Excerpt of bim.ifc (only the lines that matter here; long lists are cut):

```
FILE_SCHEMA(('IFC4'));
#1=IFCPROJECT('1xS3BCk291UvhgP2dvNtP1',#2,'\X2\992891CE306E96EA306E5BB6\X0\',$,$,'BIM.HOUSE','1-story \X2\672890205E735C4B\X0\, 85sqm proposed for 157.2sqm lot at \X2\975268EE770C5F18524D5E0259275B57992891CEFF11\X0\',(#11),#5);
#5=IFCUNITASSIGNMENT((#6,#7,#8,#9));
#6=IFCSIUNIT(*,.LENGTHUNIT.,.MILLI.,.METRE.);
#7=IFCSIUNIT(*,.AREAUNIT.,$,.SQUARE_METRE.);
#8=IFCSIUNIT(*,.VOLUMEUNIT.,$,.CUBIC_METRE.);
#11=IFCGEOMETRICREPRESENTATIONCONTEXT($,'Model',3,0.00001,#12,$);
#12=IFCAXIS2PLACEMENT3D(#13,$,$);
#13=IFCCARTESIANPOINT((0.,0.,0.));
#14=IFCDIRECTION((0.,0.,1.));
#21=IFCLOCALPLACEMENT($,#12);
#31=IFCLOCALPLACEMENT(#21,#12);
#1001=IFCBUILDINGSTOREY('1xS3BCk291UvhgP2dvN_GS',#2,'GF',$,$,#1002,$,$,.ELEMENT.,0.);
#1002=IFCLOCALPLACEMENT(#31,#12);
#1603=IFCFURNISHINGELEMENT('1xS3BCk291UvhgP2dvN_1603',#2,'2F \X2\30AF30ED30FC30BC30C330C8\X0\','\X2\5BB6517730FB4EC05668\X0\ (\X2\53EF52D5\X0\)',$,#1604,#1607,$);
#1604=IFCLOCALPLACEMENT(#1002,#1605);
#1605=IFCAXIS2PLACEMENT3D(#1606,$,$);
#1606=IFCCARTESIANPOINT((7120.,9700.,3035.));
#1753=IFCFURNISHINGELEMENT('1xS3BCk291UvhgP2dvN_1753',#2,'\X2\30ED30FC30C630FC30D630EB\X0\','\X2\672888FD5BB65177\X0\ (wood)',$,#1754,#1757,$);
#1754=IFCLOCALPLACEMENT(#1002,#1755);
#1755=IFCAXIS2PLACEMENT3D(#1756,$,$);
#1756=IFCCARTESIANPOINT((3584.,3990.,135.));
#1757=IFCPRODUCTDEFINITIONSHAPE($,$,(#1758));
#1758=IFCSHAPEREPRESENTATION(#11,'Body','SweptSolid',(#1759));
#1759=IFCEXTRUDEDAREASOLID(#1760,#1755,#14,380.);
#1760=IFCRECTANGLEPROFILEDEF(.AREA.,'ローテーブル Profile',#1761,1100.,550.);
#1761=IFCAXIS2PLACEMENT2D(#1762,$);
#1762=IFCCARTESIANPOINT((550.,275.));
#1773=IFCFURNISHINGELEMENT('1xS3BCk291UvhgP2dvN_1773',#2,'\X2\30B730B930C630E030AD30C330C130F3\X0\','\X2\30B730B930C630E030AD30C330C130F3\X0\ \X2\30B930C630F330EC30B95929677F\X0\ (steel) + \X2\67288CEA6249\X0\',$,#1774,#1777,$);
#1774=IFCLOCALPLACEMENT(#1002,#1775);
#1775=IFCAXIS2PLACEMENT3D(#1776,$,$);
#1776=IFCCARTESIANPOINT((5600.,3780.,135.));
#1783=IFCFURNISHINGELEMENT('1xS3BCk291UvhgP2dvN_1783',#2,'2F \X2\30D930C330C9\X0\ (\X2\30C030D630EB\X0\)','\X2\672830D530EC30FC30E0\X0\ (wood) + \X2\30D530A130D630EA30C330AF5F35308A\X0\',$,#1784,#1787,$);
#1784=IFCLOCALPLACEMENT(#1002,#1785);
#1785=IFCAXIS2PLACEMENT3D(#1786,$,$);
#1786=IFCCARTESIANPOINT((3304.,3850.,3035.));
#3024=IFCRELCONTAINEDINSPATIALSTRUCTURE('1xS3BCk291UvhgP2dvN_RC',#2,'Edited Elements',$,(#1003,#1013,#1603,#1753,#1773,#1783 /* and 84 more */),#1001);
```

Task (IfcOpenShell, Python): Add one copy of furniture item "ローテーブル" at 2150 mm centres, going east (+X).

```python
import numpy as np
import ifcopenshell
import ifcopenshell.api.geometry
import ifcopenshell.api.root
import ifcopenshell.util.element
import ifcopenshell.util.placement

model = ifcopenshell.open("bim.ifc")


def reuse_history(source, copy):
    """copy_class also copies each property set's owner history, people and application; keep the originals."""
    for rel in copy.IsDefinedBy:
        if rel.is_a("IfcRelDefinesByProperties") and (history := rel.RelatingPropertyDefinition.OwnerHistory):
            rel.RelatingPropertyDefinition.OwnerHistory = source.OwnerHistory
            ifcopenshell.util.element.remove_deep2(model, history)


source = model.by_id(1753)
base = ifcopenshell.util.placement.get_local_placement(source.ObjectPlacement)
step = np.array([1.0, 0.0, 0.0]) * 2150.0

for i in range(1, 2):
    copy = ifcopenshell.api.root.copy_class(model, product=source)
    copy.Representation = ifcopenshell.util.element.copy_deep(
        model, source.Representation, exclude=["IfcGeometricRepresentationContext", "IfcRepresentationMap"]
    )
    reuse_history(source, copy)
    matrix = base.copy()
    matrix[:3, 3] += i * step
    print("added at", matrix[:3, 3].round(3) + 0.0)
    ifcopenshell.api.geometry.edit_object_placement(model, product=copy, matrix=matrix, is_si=False)

model.write("bim_v2.ifc")
```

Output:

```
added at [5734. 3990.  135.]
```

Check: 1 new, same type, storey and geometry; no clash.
